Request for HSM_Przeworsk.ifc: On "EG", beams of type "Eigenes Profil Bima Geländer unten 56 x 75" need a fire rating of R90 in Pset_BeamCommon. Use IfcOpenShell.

First a look at what the model holds.

```python
import ifcopenshell
import ifcopenshell.util.element

model = ifcopenshell.open("HSM_Przeworsk.ifc")
print(model.schema)
storey = next(s for s in model.by_type("IfcBuildingStorey") if s.Name == "EG")
beams = [e for e in ifcopenshell.util.element.get_decomposition(storey) if e.is_a("IfcBeam")]
seen = {}
for e in beams:
    element_type = ifcopenshell.util.element.get_type(e)
    key = (element_type.Name if element_type != e and element_type else None, ifcopenshell.util.element.get_pset(e, "Pset_BeamCommon", "FireRating"))
    seen[key] = seen.get(key, 0) + 1
for (name, value), count in sorted(seen.items(), key=str):
    print(count, "x", name, "|", value)
```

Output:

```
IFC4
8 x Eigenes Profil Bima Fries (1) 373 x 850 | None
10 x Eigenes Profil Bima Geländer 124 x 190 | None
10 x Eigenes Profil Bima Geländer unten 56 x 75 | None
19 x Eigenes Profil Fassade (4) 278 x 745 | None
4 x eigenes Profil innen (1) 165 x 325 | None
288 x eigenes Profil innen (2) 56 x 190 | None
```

```python
import ifcopenshell
import ifcopenshell.api.pset
import ifcopenshell.util.element

model = ifcopenshell.open("HSM_Przeworsk.ifc")

storey = next(s for s in model.by_type("IfcBuildingStorey") if s.Name == "EG")
beams = [e for e in ifcopenshell.util.element.get_decomposition(storey) if e.is_a("IfcBeam")]

count = 0
for e in beams:
    element_type = ifcopenshell.util.element.get_type(e)
    if element_type in (None, e) or element_type.Name != "Eigenes Profil Bima Geländer unten 56 x 75":
        continue
    # add_pset returns the element's existing set when there is one.
    pset = ifcopenshell.api.pset.add_pset(model, product=e, name="Pset_BeamCommon")
    ifcopenshell.api.pset.edit_pset(model, pset=pset, properties={"FireRating": "R90"})
    count += 1

print(count, "beams updated")

model.write("HSM_Przeworsk_updated.ifc")
```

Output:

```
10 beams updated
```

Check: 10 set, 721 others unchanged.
